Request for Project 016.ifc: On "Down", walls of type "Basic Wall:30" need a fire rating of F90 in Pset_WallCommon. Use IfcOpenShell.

First a look at what the model holds.

```python
import ifcopenshell
import ifcopenshell.util.element

model = ifcopenshell.open("Project 016.ifc")
print(model.schema)
storey = next(s for s in model.by_type("IfcBuildingStorey") if s.Name == "Down")
walls = [e for e in ifcopenshell.util.element.get_decomposition(storey) if e.is_a("IfcWall")]
seen = {}
for e in walls:
    element_type = ifcopenshell.util.element.get_type(e)
    key = (element_type.Name if element_type != e and element_type else None, ifcopenshell.util.element.get_pset(e, "Pset_WallCommon", "FireRating"))
    seen[key] = seen.get(key, 0) + 1
for (name, value), count in sorted(seen.items(), key=str):
    print(count, "x", name, "|", value)
```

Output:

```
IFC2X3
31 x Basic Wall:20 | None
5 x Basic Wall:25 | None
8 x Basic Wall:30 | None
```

```python
import ifcopenshell
import ifcopenshell.api.pset
import ifcopenshell.util.element

model = ifcopenshell.open("Project 016.ifc")

storey = next(s for s in model.by_type("IfcBuildingStorey") if s.Name == "Down")
walls = [e for e in ifcopenshell.util.element.get_decomposition(storey) if e.is_a("IfcWall")]

count = 0
for e in walls:
    element_type = ifcopenshell.util.element.get_type(e)
    if element_type in (None, e) or element_type.Name != "Basic Wall:30":
        continue
    # add_pset returns the element's existing set when there is one.
    pset = ifcopenshell.api.pset.add_pset(model, product=e, name="Pset_WallCommon")
    ifcopenshell.api.pset.edit_pset(model, pset=pset, properties={"FireRating": "F90"})
    count += 1

print(count, "walls updated")

model.write("Project 016_edited.ifc")
```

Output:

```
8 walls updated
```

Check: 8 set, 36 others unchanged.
